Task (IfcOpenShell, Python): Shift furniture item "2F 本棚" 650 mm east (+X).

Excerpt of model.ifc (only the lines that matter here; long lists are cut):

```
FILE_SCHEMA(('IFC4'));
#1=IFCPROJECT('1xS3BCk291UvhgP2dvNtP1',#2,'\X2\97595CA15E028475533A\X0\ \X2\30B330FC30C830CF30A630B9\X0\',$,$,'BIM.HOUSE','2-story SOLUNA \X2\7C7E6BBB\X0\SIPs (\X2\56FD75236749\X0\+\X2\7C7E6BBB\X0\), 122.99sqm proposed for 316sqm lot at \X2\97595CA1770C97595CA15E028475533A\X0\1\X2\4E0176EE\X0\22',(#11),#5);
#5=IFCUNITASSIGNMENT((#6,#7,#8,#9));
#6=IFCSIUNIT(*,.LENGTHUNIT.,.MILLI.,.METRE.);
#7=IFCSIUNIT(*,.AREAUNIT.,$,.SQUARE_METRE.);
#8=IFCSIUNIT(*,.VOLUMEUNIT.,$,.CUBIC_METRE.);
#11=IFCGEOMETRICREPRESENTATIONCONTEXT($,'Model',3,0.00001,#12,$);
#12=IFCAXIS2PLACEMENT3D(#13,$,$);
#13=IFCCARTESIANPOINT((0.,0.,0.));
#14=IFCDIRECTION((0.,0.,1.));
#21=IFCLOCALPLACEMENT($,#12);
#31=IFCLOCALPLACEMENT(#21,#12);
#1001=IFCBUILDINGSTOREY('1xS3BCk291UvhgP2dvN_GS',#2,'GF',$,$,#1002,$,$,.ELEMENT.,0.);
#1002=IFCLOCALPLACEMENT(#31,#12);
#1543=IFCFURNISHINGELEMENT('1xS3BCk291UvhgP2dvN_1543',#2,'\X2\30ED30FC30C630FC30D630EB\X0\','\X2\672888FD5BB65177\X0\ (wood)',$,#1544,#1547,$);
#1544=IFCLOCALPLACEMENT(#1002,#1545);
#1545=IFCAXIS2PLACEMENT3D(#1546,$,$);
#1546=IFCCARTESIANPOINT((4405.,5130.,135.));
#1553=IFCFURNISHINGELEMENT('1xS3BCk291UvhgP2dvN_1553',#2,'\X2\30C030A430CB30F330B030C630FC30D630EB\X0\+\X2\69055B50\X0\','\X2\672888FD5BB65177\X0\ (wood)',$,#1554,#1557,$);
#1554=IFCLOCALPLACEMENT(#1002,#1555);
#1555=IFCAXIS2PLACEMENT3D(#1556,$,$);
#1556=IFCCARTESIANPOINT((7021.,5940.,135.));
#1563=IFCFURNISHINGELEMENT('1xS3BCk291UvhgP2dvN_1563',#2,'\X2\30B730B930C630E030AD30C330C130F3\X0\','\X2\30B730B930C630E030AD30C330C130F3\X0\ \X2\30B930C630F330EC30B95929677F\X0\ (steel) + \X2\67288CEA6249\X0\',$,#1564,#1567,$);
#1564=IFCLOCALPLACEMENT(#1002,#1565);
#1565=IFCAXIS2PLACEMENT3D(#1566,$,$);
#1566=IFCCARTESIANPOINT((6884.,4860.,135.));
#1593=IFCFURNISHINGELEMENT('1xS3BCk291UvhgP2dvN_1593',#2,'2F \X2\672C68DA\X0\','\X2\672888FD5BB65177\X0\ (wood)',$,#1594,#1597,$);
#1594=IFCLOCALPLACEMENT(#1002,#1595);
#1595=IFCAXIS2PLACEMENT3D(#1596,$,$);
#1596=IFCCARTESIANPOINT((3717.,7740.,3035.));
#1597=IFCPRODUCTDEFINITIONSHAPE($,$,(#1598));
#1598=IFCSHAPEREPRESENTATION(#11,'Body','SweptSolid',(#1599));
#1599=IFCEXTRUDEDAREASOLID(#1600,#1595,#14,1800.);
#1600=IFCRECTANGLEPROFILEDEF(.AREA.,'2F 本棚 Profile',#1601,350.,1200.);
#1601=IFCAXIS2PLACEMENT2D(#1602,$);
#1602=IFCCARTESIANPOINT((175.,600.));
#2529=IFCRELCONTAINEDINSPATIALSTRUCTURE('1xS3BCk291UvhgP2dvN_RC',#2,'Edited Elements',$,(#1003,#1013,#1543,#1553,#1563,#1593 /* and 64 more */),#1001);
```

```python
import ifcopenshell
import ifcopenshell.api.geometry
import ifcopenshell.util.placement
import ifcopenshell.util.unit

model = ifcopenshell.open("model.ifc")
unit_scale = ifcopenshell.util.unit.calculate_unit_scale(model)

item = model.by_guid("1xS3BCk291UvhgP2dvN_1593")
matrix = ifcopenshell.util.placement.get_local_placement(item.ObjectPlacement)
matrix[0, 3] += 0.65 / unit_scale
ifcopenshell.api.geometry.edit_object_placement(model, product=item, matrix=matrix, is_si=False)

print(ifcopenshell.util.placement.get_local_placement(item.ObjectPlacement).round(3) + 0.0)

model.write("model_rev.ifc")
```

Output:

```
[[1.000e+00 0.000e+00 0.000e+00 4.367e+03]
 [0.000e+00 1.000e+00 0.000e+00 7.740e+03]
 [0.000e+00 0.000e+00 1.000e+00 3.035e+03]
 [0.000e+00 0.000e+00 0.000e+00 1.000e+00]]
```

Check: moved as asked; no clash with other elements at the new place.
